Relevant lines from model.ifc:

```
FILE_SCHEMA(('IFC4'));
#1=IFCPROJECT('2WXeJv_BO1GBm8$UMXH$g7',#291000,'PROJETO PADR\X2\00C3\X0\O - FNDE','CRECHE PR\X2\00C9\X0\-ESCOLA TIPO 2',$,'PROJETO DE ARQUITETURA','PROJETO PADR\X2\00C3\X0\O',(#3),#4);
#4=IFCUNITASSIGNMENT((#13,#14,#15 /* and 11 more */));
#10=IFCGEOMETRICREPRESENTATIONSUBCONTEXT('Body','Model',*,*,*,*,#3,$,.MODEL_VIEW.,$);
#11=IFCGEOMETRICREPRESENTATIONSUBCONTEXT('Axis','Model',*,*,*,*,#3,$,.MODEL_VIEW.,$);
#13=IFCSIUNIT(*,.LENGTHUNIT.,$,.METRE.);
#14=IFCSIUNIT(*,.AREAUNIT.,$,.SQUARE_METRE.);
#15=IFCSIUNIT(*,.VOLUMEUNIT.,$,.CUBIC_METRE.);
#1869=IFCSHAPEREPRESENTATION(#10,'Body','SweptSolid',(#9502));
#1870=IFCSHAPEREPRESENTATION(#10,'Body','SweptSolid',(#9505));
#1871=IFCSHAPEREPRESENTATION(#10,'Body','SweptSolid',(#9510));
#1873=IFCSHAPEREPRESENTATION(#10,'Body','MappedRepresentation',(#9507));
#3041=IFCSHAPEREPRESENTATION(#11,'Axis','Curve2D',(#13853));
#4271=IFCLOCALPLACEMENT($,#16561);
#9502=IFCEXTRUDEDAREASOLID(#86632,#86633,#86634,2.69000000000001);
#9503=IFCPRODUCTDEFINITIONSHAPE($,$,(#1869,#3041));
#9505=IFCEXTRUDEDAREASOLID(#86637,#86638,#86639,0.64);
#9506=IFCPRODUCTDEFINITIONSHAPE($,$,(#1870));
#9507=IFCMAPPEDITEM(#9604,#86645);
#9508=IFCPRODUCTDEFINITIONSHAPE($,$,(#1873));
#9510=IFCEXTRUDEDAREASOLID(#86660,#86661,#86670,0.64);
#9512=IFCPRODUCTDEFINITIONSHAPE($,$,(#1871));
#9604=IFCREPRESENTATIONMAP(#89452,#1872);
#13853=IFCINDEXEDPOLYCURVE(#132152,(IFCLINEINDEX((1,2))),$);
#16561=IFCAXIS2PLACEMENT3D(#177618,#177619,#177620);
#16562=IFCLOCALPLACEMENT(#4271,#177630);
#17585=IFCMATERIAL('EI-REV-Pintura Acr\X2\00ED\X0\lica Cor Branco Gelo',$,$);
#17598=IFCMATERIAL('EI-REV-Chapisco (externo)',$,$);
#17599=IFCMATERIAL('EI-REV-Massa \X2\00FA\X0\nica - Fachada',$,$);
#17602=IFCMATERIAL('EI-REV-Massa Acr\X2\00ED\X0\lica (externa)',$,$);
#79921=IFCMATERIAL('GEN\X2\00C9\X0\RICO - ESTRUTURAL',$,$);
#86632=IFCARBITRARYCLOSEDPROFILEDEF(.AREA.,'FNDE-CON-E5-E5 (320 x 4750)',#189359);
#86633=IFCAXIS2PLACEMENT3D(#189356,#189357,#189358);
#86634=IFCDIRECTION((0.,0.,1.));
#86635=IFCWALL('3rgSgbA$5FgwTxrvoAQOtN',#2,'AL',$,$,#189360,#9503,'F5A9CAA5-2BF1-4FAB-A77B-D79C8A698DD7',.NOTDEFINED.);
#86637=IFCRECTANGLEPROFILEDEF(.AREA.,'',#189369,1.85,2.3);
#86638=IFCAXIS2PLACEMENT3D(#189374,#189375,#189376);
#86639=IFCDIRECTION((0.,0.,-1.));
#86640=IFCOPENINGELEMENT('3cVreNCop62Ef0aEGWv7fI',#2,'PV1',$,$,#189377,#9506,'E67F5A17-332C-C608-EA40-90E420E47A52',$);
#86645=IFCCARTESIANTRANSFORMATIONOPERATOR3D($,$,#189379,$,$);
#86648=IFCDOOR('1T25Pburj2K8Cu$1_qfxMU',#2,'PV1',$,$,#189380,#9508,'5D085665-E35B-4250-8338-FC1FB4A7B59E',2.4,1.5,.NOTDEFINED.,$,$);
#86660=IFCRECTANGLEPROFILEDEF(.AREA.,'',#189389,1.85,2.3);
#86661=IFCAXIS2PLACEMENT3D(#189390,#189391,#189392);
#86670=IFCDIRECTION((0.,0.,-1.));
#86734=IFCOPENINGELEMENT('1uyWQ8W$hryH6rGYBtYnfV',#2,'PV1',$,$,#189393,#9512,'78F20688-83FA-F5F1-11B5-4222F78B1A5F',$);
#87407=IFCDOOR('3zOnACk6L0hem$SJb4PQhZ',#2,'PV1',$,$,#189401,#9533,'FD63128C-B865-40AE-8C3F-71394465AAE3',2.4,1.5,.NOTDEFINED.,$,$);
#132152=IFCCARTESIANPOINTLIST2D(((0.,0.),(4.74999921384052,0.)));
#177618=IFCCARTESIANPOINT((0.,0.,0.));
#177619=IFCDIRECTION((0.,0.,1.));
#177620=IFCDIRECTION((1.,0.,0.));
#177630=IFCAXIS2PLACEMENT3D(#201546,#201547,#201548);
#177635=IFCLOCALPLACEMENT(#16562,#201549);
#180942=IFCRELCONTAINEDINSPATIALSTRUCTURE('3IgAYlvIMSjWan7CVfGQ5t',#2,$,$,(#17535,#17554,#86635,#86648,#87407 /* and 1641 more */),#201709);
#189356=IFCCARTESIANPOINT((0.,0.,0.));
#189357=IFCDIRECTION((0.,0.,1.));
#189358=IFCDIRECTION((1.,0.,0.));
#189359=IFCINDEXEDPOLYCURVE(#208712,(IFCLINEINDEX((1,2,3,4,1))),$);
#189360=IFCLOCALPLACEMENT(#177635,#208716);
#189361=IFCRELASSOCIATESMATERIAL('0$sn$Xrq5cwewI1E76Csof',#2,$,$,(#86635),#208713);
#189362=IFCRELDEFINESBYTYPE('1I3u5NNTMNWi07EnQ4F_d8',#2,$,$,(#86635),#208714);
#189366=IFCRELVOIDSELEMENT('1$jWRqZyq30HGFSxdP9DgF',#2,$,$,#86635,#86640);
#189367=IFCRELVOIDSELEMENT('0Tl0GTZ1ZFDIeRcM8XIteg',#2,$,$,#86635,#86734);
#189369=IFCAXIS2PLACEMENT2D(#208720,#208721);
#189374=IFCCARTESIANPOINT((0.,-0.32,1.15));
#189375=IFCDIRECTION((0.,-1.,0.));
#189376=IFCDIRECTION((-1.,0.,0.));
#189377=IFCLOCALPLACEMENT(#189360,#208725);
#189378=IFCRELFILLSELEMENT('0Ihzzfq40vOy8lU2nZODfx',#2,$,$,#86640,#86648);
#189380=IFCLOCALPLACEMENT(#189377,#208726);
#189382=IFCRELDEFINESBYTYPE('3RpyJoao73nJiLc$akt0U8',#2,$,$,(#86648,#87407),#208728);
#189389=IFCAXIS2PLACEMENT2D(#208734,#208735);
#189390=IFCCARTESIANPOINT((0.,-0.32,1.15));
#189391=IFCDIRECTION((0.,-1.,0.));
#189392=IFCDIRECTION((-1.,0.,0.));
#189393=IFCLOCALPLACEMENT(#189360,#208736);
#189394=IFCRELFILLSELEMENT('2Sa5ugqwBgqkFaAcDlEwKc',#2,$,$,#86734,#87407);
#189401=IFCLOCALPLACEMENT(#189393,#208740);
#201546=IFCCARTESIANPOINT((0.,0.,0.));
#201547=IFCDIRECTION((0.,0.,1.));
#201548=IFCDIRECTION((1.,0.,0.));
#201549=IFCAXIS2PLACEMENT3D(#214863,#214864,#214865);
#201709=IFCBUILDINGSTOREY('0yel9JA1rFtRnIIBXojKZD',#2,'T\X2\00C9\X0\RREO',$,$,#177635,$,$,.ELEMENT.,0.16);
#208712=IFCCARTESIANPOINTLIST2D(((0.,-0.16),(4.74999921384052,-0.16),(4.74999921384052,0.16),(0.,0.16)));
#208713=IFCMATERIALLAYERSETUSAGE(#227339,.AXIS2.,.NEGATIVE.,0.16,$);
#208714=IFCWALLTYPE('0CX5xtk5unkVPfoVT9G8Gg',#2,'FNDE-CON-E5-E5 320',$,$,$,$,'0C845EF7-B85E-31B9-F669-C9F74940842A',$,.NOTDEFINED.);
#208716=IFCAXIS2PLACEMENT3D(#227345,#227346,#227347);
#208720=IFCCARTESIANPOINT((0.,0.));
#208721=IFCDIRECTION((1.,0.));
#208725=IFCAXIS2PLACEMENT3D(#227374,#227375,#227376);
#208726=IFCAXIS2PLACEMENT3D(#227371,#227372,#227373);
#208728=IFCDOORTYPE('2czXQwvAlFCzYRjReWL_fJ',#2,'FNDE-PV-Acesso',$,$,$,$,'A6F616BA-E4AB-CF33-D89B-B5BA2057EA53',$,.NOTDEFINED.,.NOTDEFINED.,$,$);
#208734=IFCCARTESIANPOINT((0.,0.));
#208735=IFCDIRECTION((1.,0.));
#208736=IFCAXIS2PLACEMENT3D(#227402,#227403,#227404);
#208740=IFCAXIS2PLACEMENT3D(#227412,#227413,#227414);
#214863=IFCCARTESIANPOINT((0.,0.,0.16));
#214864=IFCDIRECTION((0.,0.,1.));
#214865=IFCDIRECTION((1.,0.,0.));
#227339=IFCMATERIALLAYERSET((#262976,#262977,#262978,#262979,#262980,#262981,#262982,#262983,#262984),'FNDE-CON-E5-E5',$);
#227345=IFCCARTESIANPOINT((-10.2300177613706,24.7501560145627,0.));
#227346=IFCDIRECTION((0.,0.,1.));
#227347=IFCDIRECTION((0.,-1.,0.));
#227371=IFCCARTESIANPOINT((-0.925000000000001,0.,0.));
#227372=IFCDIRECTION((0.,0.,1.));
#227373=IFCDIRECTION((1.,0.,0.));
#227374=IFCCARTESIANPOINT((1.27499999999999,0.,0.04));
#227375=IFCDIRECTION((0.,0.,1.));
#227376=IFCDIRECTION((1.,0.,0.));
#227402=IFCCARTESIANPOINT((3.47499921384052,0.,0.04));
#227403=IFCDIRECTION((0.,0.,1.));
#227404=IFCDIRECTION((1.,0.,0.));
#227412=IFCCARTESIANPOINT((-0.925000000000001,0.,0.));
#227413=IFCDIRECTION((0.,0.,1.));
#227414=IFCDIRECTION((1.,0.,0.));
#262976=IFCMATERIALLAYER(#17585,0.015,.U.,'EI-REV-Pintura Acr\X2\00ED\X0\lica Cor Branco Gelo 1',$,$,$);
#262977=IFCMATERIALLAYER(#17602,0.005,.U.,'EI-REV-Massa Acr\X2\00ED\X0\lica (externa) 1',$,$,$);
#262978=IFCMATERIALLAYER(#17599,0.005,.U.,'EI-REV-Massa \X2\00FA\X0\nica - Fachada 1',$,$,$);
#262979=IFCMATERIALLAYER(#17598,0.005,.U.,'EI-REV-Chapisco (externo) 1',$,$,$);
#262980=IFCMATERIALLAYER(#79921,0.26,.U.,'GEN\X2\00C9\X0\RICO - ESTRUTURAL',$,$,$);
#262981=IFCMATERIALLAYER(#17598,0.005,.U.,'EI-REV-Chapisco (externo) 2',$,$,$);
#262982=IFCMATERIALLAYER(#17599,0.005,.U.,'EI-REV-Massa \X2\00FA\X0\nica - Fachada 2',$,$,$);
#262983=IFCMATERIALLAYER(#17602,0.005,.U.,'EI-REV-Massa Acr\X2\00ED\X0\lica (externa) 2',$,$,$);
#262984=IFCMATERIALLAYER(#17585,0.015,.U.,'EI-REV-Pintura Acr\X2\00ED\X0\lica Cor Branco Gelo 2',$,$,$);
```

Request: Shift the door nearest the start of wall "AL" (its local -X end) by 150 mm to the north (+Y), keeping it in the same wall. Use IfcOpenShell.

```python
import ifcopenshell
import ifcopenshell.api.geometry
import ifcopenshell.util.placement

model = ifcopenshell.open("model.ifc")

door = model.by_id(86648)
opening = door.FillsVoids[0].RelatingOpeningElement
wall = opening.VoidsElements[0].RelatingBuildingElement

wall_matrix = ifcopenshell.util.placement.get_local_placement(wall.ObjectPlacement)
shift = wall_matrix[:3, 0] * -0.15
before = ifcopenshell.util.placement.get_local_placement(door.ObjectPlacement)[:3, 3].copy()

# The door is placed relative to its opening, so it follows when the opening moves.
matrix = ifcopenshell.util.placement.get_local_placement(opening.ObjectPlacement)
matrix[:3, 3] += shift
ifcopenshell.api.geometry.edit_object_placement(
    model, product=opening, matrix=matrix, is_si=False, should_transform_children=True
)

after = ifcopenshell.util.placement.get_local_placement(door.ObjectPlacement)[:3, 3]
print("door moved by", (after - before).round(3) + 0.0)

model.write("model-out.ifc")
```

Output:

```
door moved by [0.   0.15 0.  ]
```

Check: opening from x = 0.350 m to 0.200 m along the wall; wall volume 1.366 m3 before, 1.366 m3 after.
